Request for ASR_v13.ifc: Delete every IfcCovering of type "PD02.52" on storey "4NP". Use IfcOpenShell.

First a look at what the model holds.

```python
import ifcopenshell
import ifcopenshell.util.element

model = ifcopenshell.open("ASR_v13.ifc")
print(model.schema)
storey = next(s for s in model.by_type("IfcBuildingStorey") if s.Name == "4NP")
coverings = [e for e in ifcopenshell.util.element.get_decomposition(storey) if e.is_a("IfcCovering")]
seen = {}
for e in coverings:
    element_type = ifcopenshell.util.element.get_type(e)
    name = element_type.Name if element_type not in (None, e) else None
    seen[name] = seen.get(name, 0) + 1
for name, count in sorted(seen.items(), key=str):
    print(count, "x", name)
```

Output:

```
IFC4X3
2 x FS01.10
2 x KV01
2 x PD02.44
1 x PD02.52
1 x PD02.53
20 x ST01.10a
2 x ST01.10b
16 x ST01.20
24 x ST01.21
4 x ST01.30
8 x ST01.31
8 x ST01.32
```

```python
import ifcopenshell
import ifcopenshell.api.root
import ifcopenshell.util.element

model = ifcopenshell.open("ASR_v13.ifc")

storey = next(s for s in model.by_type("IfcBuildingStorey") if s.Name == "4NP")
coverings = [e for e in ifcopenshell.util.element.get_decomposition(storey) if e.is_a("IfcCovering")]
targets = [e for e in coverings if (t := ifcopenshell.util.element.get_type(e)) not in (None, e) and t.Name == "PD02.52"]

for e in targets:
    ifcopenshell.api.root.remove_product(model, product=e)
print(len(targets), "removed")

model.write("ASR_v13_edited.ifc")
```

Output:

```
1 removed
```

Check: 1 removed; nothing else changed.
